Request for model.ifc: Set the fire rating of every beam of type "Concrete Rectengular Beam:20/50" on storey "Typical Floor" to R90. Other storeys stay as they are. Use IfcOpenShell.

First a look at what the model holds.

```python
import ifcopenshell
import ifcopenshell.util.element

model = ifcopenshell.open("model.ifc")
print(model.schema)
storey = next(s for s in model.by_type("IfcBuildingStorey") if s.Name == "Typical Floor")
beams = [e for e in ifcopenshell.util.element.get_decomposition(storey) if e.is_a("IfcBeam")]
seen = {}
for e in beams:
    element_type = ifcopenshell.util.element.get_type(e)
    key = (element_type.Name if element_type != e and element_type else None, ifcopenshell.util.element.get_pset(e, "Pset_BeamCommon", "FireRating"))
    seen[key] = seen.get(key, 0) + 1
for (name, value), count in sorted(seen.items(), key=str):
    print(count, "x", name, "|", value)
```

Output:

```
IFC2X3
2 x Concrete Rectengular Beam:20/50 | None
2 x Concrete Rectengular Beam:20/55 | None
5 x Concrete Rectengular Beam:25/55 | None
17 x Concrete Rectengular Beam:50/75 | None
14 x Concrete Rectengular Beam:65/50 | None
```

```python
import ifcopenshell
import ifcopenshell.api.pset
import ifcopenshell.util.element

model = ifcopenshell.open("model.ifc")

storey = next(s for s in model.by_type("IfcBuildingStorey") if s.Name == "Typical Floor")
beams = [e for e in ifcopenshell.util.element.get_decomposition(storey) if e.is_a("IfcBeam")]

count = 0
for e in beams:
    element_type = ifcopenshell.util.element.get_type(e)
    if element_type in (None, e) or element_type.Name != "Concrete Rectengular Beam:20/50":
        continue
    # add_pset returns the element's existing set when there is one.
    pset = ifcopenshell.api.pset.add_pset(model, product=e, name="Pset_BeamCommon")
    ifcopenshell.api.pset.edit_pset(model, pset=pset, properties={"FireRating": "R90"})
    count += 1

print(count, "beams updated")

model.write("model-out.ifc")
```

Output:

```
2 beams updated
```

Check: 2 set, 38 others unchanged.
